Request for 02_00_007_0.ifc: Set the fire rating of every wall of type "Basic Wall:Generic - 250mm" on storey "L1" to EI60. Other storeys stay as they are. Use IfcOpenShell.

First a look at what the model holds.

```python
import ifcopenshell
import ifcopenshell.util.element

model = ifcopenshell.open("02_00_007_0.ifc")
print(model.schema)
storey = next(s for s in model.by_type("IfcBuildingStorey") if s.Name == "L1")
walls = [e for e in ifcopenshell.util.element.get_decomposition(storey) if e.is_a("IfcWall")]
seen = {}
for e in walls:
    element_type = ifcopenshell.util.element.get_type(e)
    key = (element_type.Name if element_type != e and element_type else None, ifcopenshell.util.element.get_pset(e, "Pset_WallCommon", "FireRating"))
    seen[key] = seen.get(key, 0) + 1
for (name, value), count in sorted(seen.items(), key=str):
    print(count, "x", name, "|", value)
```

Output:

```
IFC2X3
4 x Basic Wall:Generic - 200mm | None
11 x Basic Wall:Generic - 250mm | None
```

```python
import ifcopenshell
import ifcopenshell.api.pset
import ifcopenshell.util.element

model = ifcopenshell.open("02_00_007_0.ifc")

storey = next(s for s in model.by_type("IfcBuildingStorey") if s.Name == "L1")
walls = [e for e in ifcopenshell.util.element.get_decomposition(storey) if e.is_a("IfcWall")]

count = 0
for e in walls:
    element_type = ifcopenshell.util.element.get_type(e)
    if element_type in (None, e) or element_type.Name != "Basic Wall:Generic - 250mm":
        continue
    # add_pset returns the element's existing set when there is one.
    pset = ifcopenshell.api.pset.add_pset(model, product=e, name="Pset_WallCommon")
    ifcopenshell.api.pset.edit_pset(model, pset=pset, properties={"FireRating": "EI60"})
    count += 1

print(count, "walls updated")

model.write("02_00_007_0_rev.ifc")
```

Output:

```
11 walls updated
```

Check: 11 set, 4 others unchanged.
